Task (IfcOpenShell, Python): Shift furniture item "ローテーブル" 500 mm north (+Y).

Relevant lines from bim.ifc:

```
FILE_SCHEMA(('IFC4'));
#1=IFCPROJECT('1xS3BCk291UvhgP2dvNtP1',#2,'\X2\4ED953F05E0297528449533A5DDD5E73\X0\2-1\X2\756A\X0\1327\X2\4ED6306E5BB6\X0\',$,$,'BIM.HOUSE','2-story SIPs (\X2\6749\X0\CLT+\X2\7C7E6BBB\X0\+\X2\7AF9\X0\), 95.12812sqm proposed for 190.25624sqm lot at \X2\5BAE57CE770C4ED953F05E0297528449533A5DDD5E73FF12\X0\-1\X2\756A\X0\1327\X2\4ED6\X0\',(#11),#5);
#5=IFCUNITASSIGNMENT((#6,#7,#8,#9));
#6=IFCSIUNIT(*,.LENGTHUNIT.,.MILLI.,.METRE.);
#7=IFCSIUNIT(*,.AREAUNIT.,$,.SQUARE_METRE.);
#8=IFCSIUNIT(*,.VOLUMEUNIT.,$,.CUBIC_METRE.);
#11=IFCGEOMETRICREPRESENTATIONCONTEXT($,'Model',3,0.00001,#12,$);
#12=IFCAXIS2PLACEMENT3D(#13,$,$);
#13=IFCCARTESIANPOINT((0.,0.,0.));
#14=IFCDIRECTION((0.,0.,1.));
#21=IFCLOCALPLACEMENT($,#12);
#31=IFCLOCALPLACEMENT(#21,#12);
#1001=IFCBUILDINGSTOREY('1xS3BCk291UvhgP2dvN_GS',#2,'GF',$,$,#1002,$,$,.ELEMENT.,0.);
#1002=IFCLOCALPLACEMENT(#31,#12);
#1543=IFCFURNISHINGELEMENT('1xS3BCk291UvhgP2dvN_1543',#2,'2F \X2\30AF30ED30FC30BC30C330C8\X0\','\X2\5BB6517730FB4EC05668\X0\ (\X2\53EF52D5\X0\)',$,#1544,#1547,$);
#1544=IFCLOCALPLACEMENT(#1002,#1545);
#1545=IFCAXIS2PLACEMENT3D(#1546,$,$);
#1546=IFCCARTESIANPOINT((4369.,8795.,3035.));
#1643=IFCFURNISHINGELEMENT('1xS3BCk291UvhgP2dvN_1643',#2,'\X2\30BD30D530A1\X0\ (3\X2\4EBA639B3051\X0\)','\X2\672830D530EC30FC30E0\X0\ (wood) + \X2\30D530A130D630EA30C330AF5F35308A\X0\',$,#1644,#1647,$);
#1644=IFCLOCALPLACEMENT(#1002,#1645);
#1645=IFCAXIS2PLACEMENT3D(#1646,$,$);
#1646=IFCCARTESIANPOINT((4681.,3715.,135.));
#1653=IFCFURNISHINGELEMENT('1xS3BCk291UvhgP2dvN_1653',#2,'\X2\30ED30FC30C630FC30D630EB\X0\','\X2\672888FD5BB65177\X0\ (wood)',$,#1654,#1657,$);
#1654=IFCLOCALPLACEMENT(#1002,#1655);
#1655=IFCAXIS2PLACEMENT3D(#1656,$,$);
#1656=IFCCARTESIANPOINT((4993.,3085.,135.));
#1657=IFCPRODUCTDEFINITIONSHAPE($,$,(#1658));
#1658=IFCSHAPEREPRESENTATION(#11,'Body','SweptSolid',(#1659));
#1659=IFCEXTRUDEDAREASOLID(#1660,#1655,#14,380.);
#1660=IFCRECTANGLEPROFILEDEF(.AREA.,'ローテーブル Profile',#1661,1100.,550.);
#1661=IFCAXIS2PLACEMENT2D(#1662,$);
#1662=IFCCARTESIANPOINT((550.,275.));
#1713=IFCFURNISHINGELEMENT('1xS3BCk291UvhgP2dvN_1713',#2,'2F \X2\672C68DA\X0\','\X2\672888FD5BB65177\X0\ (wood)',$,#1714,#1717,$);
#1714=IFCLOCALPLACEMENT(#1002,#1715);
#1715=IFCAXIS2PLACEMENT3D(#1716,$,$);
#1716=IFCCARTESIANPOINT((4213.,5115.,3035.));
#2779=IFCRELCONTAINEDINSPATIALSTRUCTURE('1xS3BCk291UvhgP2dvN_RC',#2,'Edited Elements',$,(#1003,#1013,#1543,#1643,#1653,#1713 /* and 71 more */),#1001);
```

```python
import ifcopenshell
import ifcopenshell.api.geometry
import ifcopenshell.util.placement
import ifcopenshell.util.unit

model = ifcopenshell.open("bim.ifc")
unit_scale = ifcopenshell.util.unit.calculate_unit_scale(model)

item = model.by_guid("1xS3BCk291UvhgP2dvN_1653")
matrix = ifcopenshell.util.placement.get_local_placement(item.ObjectPlacement)
matrix[1, 3] += 0.5 / unit_scale
ifcopenshell.api.geometry.edit_object_placement(model, product=item, matrix=matrix, is_si=False)

print(ifcopenshell.util.placement.get_local_placement(item.ObjectPlacement).round(3) + 0.0)

model.write("bim_v2.ifc")
```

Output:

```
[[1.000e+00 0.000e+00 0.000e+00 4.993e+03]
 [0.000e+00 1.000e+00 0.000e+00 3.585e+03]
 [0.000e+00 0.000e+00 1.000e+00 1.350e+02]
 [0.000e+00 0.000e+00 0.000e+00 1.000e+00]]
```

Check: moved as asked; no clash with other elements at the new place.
